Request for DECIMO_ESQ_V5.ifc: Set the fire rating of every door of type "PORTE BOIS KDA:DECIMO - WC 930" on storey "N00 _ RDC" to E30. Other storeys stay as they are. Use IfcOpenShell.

First a look at what the model holds.

```python
import ifcopenshell
import ifcopenshell.util.element

model = ifcopenshell.open("DECIMO_ESQ_V5.ifc")
print(model.schema)
storey = next(s for s in model.by_type("IfcBuildingStorey") if s.Name == "N00 _ RDC")
doors = [e for e in ifcopenshell.util.element.get_decomposition(storey) if e.is_a("IfcDoor")]
seen = {}
for e in doors:
    element_type = ifcopenshell.util.element.get_type(e)
    key = (element_type.Name if element_type != e and element_type else None, ifcopenshell.util.element.get_pset(e, "Pset_DoorCommon", "FireRating"))
    seen[key] = seen.get(key, 0) + 1
for (name, value), count in sorted(seen.items(), key=str):
    print(count, "x", name, "|", value)
```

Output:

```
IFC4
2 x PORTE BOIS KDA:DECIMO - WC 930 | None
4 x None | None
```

```python
import ifcopenshell
import ifcopenshell.api.pset
import ifcopenshell.util.element

model = ifcopenshell.open("DECIMO_ESQ_V5.ifc")

storey = next(s for s in model.by_type("IfcBuildingStorey") if s.Name == "N00 _ RDC")
doors = [e for e in ifcopenshell.util.element.get_decomposition(storey) if e.is_a("IfcDoor")]

count = 0
for e in doors:
    element_type = ifcopenshell.util.element.get_type(e)
    if element_type in (None, e) or element_type.Name != "PORTE BOIS KDA:DECIMO - WC 930":
        continue
    # add_pset returns the element's existing set when there is one.
    pset = ifcopenshell.api.pset.add_pset(model, product=e, name="Pset_DoorCommon")
    ifcopenshell.api.pset.edit_pset(model, pset=pset, properties={"FireRating": "E30"})
    count += 1

print(count, "doors updated")

model.write("DECIMO_ESQ_V5-out.ifc")
```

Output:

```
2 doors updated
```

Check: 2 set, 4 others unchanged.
